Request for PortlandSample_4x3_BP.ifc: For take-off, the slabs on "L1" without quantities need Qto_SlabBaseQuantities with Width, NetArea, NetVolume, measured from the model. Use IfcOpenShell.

First a look at what the model holds.

```python
import ifcopenshell
import ifcopenshell.util.element
import ifcopenshell.util.unit

model = ifcopenshell.open("PortlandSample_4x3_BP.ifc")
print(model.schema)
for unit_type in ("LENGTHUNIT", "AREAUNIT", "VOLUMEUNIT"):
    print(unit_type, ifcopenshell.util.unit.calculate_unit_scale(model, unit_type))
storey = next(s for s in model.by_type("IfcBuildingStorey") if s.Name == "L1")
slabs = [e for e in ifcopenshell.util.element.get_decomposition(storey) if e.is_a("IfcSlab")]
for e in sorted(slabs, key=lambda e: e.id()):
    print(e.id(), e.is_a(), e.Name, list(ifcopenshell.util.element.get_psets(e, qtos_only=True)), sep=" | ")
```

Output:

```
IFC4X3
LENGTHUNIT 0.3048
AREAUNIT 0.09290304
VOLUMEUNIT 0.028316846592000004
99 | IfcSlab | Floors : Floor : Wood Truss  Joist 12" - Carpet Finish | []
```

```python
import ifcopenshell
import ifcopenshell.api.pset
import ifcopenshell.geom
import ifcopenshell.util.element
import ifcopenshell.util.shape
import ifcopenshell.util.unit

model = ifcopenshell.open("PortlandSample_4x3_BP.ifc")
unit_scale = ifcopenshell.util.unit.calculate_unit_scale(model)
area_scale = ifcopenshell.util.unit.calculate_unit_scale(model, "AREAUNIT")
volume_scale = ifcopenshell.util.unit.calculate_unit_scale(model, "VOLUMEUNIT")
settings = ifcopenshell.geom.settings()

storey = next(s for s in model.by_type("IfcBuildingStorey") if s.Name == "L1")
slabs = [e for e in ifcopenshell.util.element.get_decomposition(storey) if e.is_a("IfcSlab")]

for e in sorted(slabs, key=lambda e: e.id()):
    if ifcopenshell.util.element.get_psets(e, qtos_only=True, should_inherit=False):
        continue
    # Geometry comes back in metres, in the element's own axes.
    shape = ifcopenshell.geom.create_shape(settings, e)
    values = {
        "Width": ifcopenshell.util.shape.get_z(shape.geometry) / unit_scale,
        "NetArea": ifcopenshell.util.shape.get_footprint_area(shape.geometry) / area_scale,
        "NetVolume": ifcopenshell.util.shape.get_volume(shape.geometry) / volume_scale,
    }
    qto = ifcopenshell.api.pset.add_qto(model, product=e, name="Qto_SlabBaseQuantities")
    ifcopenshell.api.pset.edit_qto(model, qto=qto, properties=values)
    print(e.id(), {k: round(v, 3) for k, v in values.items()})

model.write("PortlandSample_4x3_BP_updated.ifc")
```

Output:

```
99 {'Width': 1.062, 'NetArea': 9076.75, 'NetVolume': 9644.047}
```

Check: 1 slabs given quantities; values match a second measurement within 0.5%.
